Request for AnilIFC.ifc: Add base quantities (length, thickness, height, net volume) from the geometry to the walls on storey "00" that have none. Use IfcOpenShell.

First a look at what the model holds.

```python
import ifcopenshell
import ifcopenshell.util.element
import ifcopenshell.util.unit

model = ifcopenshell.open("AnilIFC.ifc")
print(model.schema)
for unit_type in ("LENGTHUNIT", "AREAUNIT", "VOLUMEUNIT"):
    print(unit_type, ifcopenshell.util.unit.calculate_unit_scale(model, unit_type))
storey = next(s for s in model.by_type("IfcBuildingStorey") if s.Name == "00")
walls = [e for e in ifcopenshell.util.element.get_decomposition(storey) if e.is_a("IfcWall")]
for e in sorted(walls, key=lambda e: e.id()):
    print(e.id(), e.is_a(), e.Name, list(ifcopenshell.util.element.get_psets(e, qtos_only=True)), sep=" | ")
```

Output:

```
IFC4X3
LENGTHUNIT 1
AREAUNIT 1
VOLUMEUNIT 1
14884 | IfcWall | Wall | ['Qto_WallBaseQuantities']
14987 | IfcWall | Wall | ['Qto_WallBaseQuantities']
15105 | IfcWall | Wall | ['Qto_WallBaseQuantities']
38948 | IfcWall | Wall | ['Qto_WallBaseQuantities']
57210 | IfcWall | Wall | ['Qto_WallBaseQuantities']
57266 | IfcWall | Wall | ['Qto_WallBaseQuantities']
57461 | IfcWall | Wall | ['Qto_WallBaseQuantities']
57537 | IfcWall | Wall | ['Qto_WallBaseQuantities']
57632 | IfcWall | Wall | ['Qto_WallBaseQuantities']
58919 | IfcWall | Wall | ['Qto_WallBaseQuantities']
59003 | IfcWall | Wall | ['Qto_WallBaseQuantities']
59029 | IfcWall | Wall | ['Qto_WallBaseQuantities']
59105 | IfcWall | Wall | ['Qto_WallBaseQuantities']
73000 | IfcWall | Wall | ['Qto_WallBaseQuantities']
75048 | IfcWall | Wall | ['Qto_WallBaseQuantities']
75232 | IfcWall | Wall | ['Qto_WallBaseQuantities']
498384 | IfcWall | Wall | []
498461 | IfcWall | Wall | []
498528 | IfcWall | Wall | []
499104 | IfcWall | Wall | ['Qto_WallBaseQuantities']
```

```python
import ifcopenshell
import ifcopenshell.api.pset
import ifcopenshell.geom
import ifcopenshell.util.element
import ifcopenshell.util.shape
import ifcopenshell.util.unit

model = ifcopenshell.open("AnilIFC.ifc")
unit_scale = ifcopenshell.util.unit.calculate_unit_scale(model)
volume_scale = ifcopenshell.util.unit.calculate_unit_scale(model, "VOLUMEUNIT")
settings = ifcopenshell.geom.settings()

storey = next(s for s in model.by_type("IfcBuildingStorey") if s.Name == "00")
walls = [e for e in ifcopenshell.util.element.get_decomposition(storey) if e.is_a("IfcWall")]

for e in sorted(walls, key=lambda e: e.id()):
    if ifcopenshell.util.element.get_psets(e, qtos_only=True, should_inherit=False):
        continue
    # Geometry comes back in metres, in the element's own axes.
    shape = ifcopenshell.geom.create_shape(settings, e)
    values = {
        "Length": ifcopenshell.util.shape.get_x(shape.geometry) / unit_scale,
        "Width": ifcopenshell.util.shape.get_y(shape.geometry) / unit_scale,
        "Height": ifcopenshell.util.shape.get_z(shape.geometry) / unit_scale,
        "NetVolume": ifcopenshell.util.shape.get_volume(shape.geometry) / volume_scale,
    }
    qto = ifcopenshell.api.pset.add_qto(model, product=e, name="Qto_WallBaseQuantities")
    ifcopenshell.api.pset.edit_qto(model, qto=qto, properties=values)
    print(e.id(), {k: round(v, 3) for k, v in values.items()})

model.write("AnilIFC_v2.ifc")
```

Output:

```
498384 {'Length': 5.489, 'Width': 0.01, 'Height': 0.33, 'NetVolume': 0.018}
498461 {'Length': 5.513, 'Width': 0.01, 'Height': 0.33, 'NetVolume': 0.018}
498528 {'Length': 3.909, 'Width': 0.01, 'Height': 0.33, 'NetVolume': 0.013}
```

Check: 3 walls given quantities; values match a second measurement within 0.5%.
